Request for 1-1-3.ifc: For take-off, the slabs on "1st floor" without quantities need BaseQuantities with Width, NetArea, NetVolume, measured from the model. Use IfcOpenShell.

First a look at what the model holds.

```python
import ifcopenshell
import ifcopenshell.util.element
import ifcopenshell.util.unit

model = ifcopenshell.open("1-1-3.ifc")
print(model.schema)
for unit_type in ("LENGTHUNIT", "AREAUNIT", "VOLUMEUNIT"):
    print(unit_type, ifcopenshell.util.unit.calculate_unit_scale(model, unit_type))
storey = next(s for s in model.by_type("IfcBuildingStorey") if s.Name == "1st floor")
slabs = [e for e in ifcopenshell.util.element.get_decomposition(storey) if e.is_a("IfcSlab")]
for e in sorted(slabs, key=lambda e: e.id()):
    print(e.id(), e.is_a(), e.Name, list(ifcopenshell.util.element.get_psets(e, qtos_only=True)), sep=" | ")
```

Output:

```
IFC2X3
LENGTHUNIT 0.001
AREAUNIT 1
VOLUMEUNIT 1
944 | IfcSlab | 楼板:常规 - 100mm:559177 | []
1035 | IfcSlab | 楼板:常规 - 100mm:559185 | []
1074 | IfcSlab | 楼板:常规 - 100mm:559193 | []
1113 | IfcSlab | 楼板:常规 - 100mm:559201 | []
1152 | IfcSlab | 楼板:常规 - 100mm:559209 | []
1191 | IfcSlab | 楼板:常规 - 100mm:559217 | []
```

```python
import ifcopenshell
import ifcopenshell.api.pset
import ifcopenshell.geom
import ifcopenshell.util.element
import ifcopenshell.util.shape
import ifcopenshell.util.unit

model = ifcopenshell.open("1-1-3.ifc")
unit_scale = ifcopenshell.util.unit.calculate_unit_scale(model)
area_scale = ifcopenshell.util.unit.calculate_unit_scale(model, "AREAUNIT")
volume_scale = ifcopenshell.util.unit.calculate_unit_scale(model, "VOLUMEUNIT")
settings = ifcopenshell.geom.settings()

storey = next(s for s in model.by_type("IfcBuildingStorey") if s.Name == "1st floor")
slabs = [e for e in ifcopenshell.util.element.get_decomposition(storey) if e.is_a("IfcSlab")]

for e in sorted(slabs, key=lambda e: e.id()):
    if ifcopenshell.util.element.get_psets(e, qtos_only=True, should_inherit=False):
        continue
    # Geometry comes back in metres, in the element's own axes.
    shape = ifcopenshell.geom.create_shape(settings, e)
    values = {
        "Width": ifcopenshell.util.shape.get_z(shape.geometry) / unit_scale,
        "NetArea": ifcopenshell.util.shape.get_footprint_area(shape.geometry) / area_scale,
        "NetVolume": ifcopenshell.util.shape.get_volume(shape.geometry) / volume_scale,
    }
    qto = ifcopenshell.api.pset.add_qto(model, product=e, name="BaseQuantities")
    ifcopenshell.api.pset.edit_qto(model, qto=qto, properties=values)
    print(e.id(), {k: round(v, 3) for k, v in values.items()})

model.write("1-1-3-out.ifc")
```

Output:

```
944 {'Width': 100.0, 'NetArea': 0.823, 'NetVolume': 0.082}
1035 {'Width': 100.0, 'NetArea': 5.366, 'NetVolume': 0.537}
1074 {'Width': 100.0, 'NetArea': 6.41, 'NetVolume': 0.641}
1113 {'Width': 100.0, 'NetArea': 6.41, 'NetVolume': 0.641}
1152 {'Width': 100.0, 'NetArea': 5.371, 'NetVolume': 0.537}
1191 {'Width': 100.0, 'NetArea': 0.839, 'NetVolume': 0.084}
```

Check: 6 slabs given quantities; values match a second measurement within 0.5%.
